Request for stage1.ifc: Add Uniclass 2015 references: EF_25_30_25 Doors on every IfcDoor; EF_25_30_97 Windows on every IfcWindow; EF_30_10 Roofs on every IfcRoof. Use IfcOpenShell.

First a look at what the model holds.

```python
import ifcopenshell

model = ifcopenshell.open("stage1.ifc")
print(model.schema)
print("classifications:", [c.Name for c in model.by_type("IfcClassification")])
for ifc_class in ("IfcDoor", "IfcRoof", "IfcStair", "IfcWall", "IfcWindow"):
    print(ifc_class, len(model.by_type(ifc_class)))
```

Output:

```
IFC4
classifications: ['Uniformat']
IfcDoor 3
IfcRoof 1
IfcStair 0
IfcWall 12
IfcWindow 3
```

```python
import ifcopenshell
import ifcopenshell.api.classification

model = ifcopenshell.open("stage1.ifc")

system = ifcopenshell.api.classification.add_classification(model, classification="Uniclass 2015")

codes = {
    "IfcDoor": ("EF_25_30_25", "Doors"),
    "IfcWindow": ("EF_25_30_97", "Windows"),
    "IfcRoof": ("EF_30_10", "Roofs"),
}
for ifc_class, (code, name) in codes.items():
    products = model.by_type(ifc_class)
    ifcopenshell.api.classification.add_reference(
        model, products=products, classification=system, identification=code, name=name
    )
    print(code, len(products))

model.write("stage1-out.ifc")
```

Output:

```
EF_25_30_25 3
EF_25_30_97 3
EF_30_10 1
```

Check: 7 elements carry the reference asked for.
